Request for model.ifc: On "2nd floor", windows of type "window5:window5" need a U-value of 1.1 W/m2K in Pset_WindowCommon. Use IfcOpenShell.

First a look at what the model holds.

```python
import ifcopenshell
import ifcopenshell.util.element

model = ifcopenshell.open("model.ifc")
print(model.schema)
storey = next(s for s in model.by_type("IfcBuildingStorey") if s.Name == "2nd floor")
windows = [e for e in ifcopenshell.util.element.get_decomposition(storey) if e.is_a("IfcWindow")]
seen = {}
for e in windows:
    element_type = ifcopenshell.util.element.get_type(e)
    key = (element_type.Name if element_type != e and element_type else None, ifcopenshell.util.element.get_pset(e, "Pset_WindowCommon", "ThermalTransmittance"))
    seen[key] = seen.get(key, 0) + 1
for (name, value), count in sorted(seen.items(), key=str):
    print(count, "x", name, "|", value)
```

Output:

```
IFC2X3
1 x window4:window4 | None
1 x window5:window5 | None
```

```python
import ifcopenshell
import ifcopenshell.api.pset
import ifcopenshell.util.element

model = ifcopenshell.open("model.ifc")

storey = next(s for s in model.by_type("IfcBuildingStorey") if s.Name == "2nd floor")
windows = [e for e in ifcopenshell.util.element.get_decomposition(storey) if e.is_a("IfcWindow")]

count = 0
for e in windows:
    element_type = ifcopenshell.util.element.get_type(e)
    if element_type in (None, e) or element_type.Name != "window5:window5":
        continue
    # add_pset returns the element's existing set when there is one.
    pset = ifcopenshell.api.pset.add_pset(model, product=e, name="Pset_WindowCommon")
    ifcopenshell.api.pset.edit_pset(model, pset=pset, properties={"ThermalTransmittance": 1.1})
    count += 1

print(count, "windows updated")

model.write("model_v2.ifc")
```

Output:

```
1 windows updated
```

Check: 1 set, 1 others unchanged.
